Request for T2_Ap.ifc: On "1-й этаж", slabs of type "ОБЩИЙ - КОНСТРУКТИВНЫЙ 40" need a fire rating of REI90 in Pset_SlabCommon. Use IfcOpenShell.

First a look at what the model holds.

```python
import ifcopenshell
import ifcopenshell.util.element

model = ifcopenshell.open("T2_Ap.ifc")
print(model.schema)
storey = next(s for s in model.by_type("IfcBuildingStorey") if s.Name == "1-й этаж")
slabs = [e for e in ifcopenshell.util.element.get_decomposition(storey) if e.is_a("IfcSlab")]
seen = {}
for e in slabs:
    element_type = ifcopenshell.util.element.get_type(e)
    key = (element_type.Name if element_type != e and element_type else None, ifcopenshell.util.element.get_pset(e, "Pset_SlabCommon", "FireRating"))
    seen[key] = seen.get(key, 0) + 1
for (name, value), count in sorted(seen.items(), key=str):
    print(count, "x", name, "|", value)
```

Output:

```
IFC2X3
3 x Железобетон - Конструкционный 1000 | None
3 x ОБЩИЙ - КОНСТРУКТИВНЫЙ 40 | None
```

```python
import ifcopenshell
import ifcopenshell.api.pset
import ifcopenshell.util.element

model = ifcopenshell.open("T2_Ap.ifc")

storey = next(s for s in model.by_type("IfcBuildingStorey") if s.Name == "1-й этаж")
slabs = [e for e in ifcopenshell.util.element.get_decomposition(storey) if e.is_a("IfcSlab")]

count = 0
for e in slabs:
    element_type = ifcopenshell.util.element.get_type(e)
    if element_type in (None, e) or element_type.Name != "ОБЩИЙ - КОНСТРУКТИВНЫЙ 40":
        continue
    # add_pset returns the element's existing set when there is one.
    pset = ifcopenshell.api.pset.add_pset(model, product=e, name="Pset_SlabCommon")
    ifcopenshell.api.pset.edit_pset(model, pset=pset, properties={"FireRating": "REI90"})
    count += 1

print(count, "slabs updated")

model.write("T2_Ap_v2.ifc")
```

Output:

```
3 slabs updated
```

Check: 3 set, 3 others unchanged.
